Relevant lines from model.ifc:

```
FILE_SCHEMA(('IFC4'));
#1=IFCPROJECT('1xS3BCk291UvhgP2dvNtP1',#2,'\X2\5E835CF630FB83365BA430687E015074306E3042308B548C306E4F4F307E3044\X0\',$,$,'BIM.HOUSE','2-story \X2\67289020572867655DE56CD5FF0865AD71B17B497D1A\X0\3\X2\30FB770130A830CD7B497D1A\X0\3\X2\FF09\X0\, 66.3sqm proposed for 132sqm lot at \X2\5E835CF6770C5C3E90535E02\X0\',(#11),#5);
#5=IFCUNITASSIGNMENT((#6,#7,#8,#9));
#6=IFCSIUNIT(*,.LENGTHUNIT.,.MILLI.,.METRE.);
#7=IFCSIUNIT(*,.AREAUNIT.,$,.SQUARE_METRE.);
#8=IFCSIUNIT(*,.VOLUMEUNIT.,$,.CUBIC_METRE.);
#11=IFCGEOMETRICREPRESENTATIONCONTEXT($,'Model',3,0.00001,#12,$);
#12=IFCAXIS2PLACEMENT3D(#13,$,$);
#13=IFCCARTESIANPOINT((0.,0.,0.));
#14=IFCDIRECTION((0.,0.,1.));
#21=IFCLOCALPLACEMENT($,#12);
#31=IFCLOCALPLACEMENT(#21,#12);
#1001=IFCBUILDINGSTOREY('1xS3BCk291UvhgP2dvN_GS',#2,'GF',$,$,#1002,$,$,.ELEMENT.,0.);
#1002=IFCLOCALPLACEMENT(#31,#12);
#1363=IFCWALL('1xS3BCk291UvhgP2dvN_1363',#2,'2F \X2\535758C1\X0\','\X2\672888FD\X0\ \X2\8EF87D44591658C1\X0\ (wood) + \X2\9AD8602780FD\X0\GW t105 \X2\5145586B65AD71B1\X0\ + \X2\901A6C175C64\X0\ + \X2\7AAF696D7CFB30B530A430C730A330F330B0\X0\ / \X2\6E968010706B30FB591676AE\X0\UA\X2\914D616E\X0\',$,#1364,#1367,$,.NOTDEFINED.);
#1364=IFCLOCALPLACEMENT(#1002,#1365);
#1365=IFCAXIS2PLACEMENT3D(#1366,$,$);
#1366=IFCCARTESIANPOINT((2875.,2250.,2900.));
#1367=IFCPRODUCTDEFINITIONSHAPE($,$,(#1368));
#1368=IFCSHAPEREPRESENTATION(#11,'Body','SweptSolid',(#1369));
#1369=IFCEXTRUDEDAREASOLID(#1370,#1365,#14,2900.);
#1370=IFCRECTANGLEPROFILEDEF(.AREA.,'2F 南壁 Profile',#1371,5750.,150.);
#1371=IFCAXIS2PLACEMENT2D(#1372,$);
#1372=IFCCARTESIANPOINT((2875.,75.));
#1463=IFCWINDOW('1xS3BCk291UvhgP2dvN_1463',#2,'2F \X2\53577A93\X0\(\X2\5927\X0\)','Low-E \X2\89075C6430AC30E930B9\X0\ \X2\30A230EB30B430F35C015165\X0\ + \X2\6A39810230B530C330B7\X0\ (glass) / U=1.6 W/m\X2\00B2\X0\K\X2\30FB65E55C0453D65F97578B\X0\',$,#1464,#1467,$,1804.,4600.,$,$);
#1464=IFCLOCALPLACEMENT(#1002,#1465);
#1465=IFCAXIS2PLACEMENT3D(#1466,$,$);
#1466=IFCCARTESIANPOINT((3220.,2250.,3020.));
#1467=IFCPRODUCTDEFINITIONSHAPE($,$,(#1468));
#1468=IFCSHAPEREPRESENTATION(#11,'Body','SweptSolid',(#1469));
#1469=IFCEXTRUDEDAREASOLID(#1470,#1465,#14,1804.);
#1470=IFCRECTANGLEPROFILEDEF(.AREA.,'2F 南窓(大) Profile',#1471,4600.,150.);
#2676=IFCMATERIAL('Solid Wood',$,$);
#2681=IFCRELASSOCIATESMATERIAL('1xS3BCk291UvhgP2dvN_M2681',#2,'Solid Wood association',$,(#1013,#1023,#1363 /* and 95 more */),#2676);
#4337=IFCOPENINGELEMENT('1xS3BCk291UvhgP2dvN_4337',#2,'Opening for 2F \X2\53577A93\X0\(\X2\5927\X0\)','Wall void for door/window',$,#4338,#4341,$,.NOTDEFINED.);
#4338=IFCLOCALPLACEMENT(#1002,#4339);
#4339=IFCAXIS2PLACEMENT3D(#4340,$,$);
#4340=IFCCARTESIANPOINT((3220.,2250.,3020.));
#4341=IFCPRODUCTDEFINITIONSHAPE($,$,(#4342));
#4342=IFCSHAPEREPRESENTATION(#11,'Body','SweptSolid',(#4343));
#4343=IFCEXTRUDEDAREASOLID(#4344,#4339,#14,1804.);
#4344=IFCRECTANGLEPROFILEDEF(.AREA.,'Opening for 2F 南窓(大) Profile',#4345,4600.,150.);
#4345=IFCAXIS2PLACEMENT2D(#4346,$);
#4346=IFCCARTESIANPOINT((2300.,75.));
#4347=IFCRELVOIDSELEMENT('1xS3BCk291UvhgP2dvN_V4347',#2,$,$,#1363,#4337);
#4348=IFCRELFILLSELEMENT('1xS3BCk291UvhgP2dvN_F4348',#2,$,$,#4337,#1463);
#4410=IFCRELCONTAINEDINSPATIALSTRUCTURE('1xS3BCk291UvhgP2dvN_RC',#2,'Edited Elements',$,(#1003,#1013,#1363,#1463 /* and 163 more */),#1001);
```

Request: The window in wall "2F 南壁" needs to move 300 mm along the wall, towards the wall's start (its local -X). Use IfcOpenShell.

```python
import ifcopenshell
import ifcopenshell.api.geometry
import ifcopenshell.util.placement
import ifcopenshell.util.unit

model = ifcopenshell.open("model.ifc")
unit_scale = ifcopenshell.util.unit.calculate_unit_scale(model)

window = model.by_guid("1xS3BCk291UvhgP2dvN_1463")
opening = window.FillsVoids[0].RelatingOpeningElement
wall = opening.VoidsElements[0].RelatingBuildingElement

wall_matrix = ifcopenshell.util.placement.get_local_placement(wall.ObjectPlacement)
shift = wall_matrix[:3, 0] * -0.3 / unit_scale
before = ifcopenshell.util.placement.get_local_placement(window.ObjectPlacement)[:3, 3].copy()

# The window is not placed relative to its opening, so move both.
for product in (opening, window):
    matrix = ifcopenshell.util.placement.get_local_placement(product.ObjectPlacement)
    matrix[:3, 3] += shift
    ifcopenshell.api.geometry.edit_object_placement(model, product=product, matrix=matrix, is_si=False)

after = ifcopenshell.util.placement.get_local_placement(window.ObjectPlacement)[:3, 3]
print("window moved by", (after - before).round(3) + 0.0)

model.write("model_v2.ifc")
```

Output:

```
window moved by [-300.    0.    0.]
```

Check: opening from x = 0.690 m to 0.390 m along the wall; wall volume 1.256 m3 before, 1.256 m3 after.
